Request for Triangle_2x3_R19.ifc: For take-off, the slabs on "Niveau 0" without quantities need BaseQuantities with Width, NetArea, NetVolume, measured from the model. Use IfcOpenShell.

First a look at what the model holds.

```python
import ifcopenshell
import ifcopenshell.util.element
import ifcopenshell.util.unit

model = ifcopenshell.open("Triangle_2x3_R19.ifc")
print(model.schema)
for unit_type in ("LENGTHUNIT", "AREAUNIT", "VOLUMEUNIT"):
    print(unit_type, ifcopenshell.util.unit.calculate_unit_scale(model, unit_type))
storey = next(s for s in model.by_type("IfcBuildingStorey") if s.Name == "Niveau 0")
slabs = [e for e in ifcopenshell.util.element.get_decomposition(storey) if e.is_a("IfcSlab")]
for e in sorted(slabs, key=lambda e: e.id()):
    print(e.id(), e.is_a(), e.Name, list(ifcopenshell.util.element.get_psets(e, qtos_only=True)), sep=" | ")
```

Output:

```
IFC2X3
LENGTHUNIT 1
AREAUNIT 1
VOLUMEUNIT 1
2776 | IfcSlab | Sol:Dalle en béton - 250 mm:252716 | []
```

```python
import ifcopenshell
import ifcopenshell.api.pset
import ifcopenshell.geom
import ifcopenshell.util.element
import ifcopenshell.util.shape
import ifcopenshell.util.unit

model = ifcopenshell.open("Triangle_2x3_R19.ifc")
unit_scale = ifcopenshell.util.unit.calculate_unit_scale(model)
area_scale = ifcopenshell.util.unit.calculate_unit_scale(model, "AREAUNIT")
volume_scale = ifcopenshell.util.unit.calculate_unit_scale(model, "VOLUMEUNIT")
settings = ifcopenshell.geom.settings()

storey = next(s for s in model.by_type("IfcBuildingStorey") if s.Name == "Niveau 0")
slabs = [e for e in ifcopenshell.util.element.get_decomposition(storey) if e.is_a("IfcSlab")]

for e in sorted(slabs, key=lambda e: e.id()):
    if ifcopenshell.util.element.get_psets(e, qtos_only=True, should_inherit=False):
        continue
    # Geometry comes back in metres, in the element's own axes.
    shape = ifcopenshell.geom.create_shape(settings, e)
    values = {
        "Width": ifcopenshell.util.shape.get_z(shape.geometry) / unit_scale,
        "NetArea": ifcopenshell.util.shape.get_footprint_area(shape.geometry) / area_scale,
        "NetVolume": ifcopenshell.util.shape.get_volume(shape.geometry) / volume_scale,
    }
    qto = ifcopenshell.api.pset.add_qto(model, product=e, name="BaseQuantities")
    ifcopenshell.api.pset.edit_qto(model, qto=qto, properties=values)
    print(e.id(), {k: round(v, 3) for k, v in values.items()})

model.write("Triangle_2x3_R19_rev.ifc")
```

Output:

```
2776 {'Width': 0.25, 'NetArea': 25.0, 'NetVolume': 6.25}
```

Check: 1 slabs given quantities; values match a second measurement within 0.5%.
